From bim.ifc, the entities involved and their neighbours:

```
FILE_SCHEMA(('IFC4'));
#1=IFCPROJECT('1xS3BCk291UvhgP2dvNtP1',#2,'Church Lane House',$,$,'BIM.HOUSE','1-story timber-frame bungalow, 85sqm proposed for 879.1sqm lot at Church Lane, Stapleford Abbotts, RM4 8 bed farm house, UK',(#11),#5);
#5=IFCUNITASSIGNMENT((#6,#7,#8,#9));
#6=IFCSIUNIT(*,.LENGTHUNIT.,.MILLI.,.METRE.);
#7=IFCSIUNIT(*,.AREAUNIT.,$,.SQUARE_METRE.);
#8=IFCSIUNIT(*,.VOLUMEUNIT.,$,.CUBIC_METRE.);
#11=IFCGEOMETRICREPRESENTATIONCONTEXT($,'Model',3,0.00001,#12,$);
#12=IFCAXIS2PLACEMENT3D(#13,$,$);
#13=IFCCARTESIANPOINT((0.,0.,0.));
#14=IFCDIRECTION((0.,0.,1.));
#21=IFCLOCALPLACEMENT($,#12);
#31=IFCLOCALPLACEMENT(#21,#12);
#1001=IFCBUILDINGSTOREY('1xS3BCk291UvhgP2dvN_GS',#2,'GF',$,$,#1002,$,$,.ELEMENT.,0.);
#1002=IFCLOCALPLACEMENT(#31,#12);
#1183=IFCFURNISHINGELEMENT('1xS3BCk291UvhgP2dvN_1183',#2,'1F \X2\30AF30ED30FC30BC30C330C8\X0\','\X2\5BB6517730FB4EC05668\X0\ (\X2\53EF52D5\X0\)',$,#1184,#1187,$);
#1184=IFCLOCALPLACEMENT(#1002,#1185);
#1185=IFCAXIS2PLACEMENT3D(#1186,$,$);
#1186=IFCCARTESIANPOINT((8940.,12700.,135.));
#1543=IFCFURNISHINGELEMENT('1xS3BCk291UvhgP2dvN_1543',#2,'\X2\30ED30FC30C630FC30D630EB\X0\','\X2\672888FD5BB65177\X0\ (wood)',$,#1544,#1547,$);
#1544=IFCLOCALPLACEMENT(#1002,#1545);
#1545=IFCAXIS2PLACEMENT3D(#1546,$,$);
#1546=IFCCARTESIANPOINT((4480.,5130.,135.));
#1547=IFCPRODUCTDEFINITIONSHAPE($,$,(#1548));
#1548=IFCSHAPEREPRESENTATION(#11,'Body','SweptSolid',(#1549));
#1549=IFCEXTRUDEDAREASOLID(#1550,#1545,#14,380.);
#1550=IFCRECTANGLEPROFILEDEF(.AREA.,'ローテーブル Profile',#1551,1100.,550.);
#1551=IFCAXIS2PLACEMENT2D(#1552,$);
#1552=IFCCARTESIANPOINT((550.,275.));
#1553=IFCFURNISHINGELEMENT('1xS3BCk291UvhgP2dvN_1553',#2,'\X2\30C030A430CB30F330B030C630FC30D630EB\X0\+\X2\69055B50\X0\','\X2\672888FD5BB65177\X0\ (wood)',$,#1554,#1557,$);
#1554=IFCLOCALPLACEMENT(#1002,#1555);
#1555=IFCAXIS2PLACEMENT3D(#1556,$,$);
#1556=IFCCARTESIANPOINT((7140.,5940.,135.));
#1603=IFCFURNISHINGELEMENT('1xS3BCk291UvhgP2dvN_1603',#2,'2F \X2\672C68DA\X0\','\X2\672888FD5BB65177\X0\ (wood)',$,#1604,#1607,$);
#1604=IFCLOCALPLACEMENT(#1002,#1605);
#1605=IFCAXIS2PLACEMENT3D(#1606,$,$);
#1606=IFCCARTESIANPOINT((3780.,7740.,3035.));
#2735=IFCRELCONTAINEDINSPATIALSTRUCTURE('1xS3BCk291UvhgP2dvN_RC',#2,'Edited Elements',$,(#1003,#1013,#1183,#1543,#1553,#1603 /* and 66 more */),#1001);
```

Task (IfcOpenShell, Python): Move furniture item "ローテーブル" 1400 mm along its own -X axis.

```python
import ifcopenshell
import ifcopenshell.api.geometry
import ifcopenshell.util.placement
import ifcopenshell.util.unit

model = ifcopenshell.open("bim.ifc")
unit_scale = ifcopenshell.util.unit.calculate_unit_scale(model)

item = model.by_guid("1xS3BCk291UvhgP2dvN_1543")
matrix = ifcopenshell.util.placement.get_local_placement(item.ObjectPlacement)
matrix[:3, 3] -= matrix[:3, 0] * 1.4 / unit_scale
ifcopenshell.api.geometry.edit_object_placement(model, product=item, matrix=matrix, is_si=False)

print(ifcopenshell.util.placement.get_local_placement(item.ObjectPlacement).round(3) + 0.0)

model.write("bim_updated.ifc")
```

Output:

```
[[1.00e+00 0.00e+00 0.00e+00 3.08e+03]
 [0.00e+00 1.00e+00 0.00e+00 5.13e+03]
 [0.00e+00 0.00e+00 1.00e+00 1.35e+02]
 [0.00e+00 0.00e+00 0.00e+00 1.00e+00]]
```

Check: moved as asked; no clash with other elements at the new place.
